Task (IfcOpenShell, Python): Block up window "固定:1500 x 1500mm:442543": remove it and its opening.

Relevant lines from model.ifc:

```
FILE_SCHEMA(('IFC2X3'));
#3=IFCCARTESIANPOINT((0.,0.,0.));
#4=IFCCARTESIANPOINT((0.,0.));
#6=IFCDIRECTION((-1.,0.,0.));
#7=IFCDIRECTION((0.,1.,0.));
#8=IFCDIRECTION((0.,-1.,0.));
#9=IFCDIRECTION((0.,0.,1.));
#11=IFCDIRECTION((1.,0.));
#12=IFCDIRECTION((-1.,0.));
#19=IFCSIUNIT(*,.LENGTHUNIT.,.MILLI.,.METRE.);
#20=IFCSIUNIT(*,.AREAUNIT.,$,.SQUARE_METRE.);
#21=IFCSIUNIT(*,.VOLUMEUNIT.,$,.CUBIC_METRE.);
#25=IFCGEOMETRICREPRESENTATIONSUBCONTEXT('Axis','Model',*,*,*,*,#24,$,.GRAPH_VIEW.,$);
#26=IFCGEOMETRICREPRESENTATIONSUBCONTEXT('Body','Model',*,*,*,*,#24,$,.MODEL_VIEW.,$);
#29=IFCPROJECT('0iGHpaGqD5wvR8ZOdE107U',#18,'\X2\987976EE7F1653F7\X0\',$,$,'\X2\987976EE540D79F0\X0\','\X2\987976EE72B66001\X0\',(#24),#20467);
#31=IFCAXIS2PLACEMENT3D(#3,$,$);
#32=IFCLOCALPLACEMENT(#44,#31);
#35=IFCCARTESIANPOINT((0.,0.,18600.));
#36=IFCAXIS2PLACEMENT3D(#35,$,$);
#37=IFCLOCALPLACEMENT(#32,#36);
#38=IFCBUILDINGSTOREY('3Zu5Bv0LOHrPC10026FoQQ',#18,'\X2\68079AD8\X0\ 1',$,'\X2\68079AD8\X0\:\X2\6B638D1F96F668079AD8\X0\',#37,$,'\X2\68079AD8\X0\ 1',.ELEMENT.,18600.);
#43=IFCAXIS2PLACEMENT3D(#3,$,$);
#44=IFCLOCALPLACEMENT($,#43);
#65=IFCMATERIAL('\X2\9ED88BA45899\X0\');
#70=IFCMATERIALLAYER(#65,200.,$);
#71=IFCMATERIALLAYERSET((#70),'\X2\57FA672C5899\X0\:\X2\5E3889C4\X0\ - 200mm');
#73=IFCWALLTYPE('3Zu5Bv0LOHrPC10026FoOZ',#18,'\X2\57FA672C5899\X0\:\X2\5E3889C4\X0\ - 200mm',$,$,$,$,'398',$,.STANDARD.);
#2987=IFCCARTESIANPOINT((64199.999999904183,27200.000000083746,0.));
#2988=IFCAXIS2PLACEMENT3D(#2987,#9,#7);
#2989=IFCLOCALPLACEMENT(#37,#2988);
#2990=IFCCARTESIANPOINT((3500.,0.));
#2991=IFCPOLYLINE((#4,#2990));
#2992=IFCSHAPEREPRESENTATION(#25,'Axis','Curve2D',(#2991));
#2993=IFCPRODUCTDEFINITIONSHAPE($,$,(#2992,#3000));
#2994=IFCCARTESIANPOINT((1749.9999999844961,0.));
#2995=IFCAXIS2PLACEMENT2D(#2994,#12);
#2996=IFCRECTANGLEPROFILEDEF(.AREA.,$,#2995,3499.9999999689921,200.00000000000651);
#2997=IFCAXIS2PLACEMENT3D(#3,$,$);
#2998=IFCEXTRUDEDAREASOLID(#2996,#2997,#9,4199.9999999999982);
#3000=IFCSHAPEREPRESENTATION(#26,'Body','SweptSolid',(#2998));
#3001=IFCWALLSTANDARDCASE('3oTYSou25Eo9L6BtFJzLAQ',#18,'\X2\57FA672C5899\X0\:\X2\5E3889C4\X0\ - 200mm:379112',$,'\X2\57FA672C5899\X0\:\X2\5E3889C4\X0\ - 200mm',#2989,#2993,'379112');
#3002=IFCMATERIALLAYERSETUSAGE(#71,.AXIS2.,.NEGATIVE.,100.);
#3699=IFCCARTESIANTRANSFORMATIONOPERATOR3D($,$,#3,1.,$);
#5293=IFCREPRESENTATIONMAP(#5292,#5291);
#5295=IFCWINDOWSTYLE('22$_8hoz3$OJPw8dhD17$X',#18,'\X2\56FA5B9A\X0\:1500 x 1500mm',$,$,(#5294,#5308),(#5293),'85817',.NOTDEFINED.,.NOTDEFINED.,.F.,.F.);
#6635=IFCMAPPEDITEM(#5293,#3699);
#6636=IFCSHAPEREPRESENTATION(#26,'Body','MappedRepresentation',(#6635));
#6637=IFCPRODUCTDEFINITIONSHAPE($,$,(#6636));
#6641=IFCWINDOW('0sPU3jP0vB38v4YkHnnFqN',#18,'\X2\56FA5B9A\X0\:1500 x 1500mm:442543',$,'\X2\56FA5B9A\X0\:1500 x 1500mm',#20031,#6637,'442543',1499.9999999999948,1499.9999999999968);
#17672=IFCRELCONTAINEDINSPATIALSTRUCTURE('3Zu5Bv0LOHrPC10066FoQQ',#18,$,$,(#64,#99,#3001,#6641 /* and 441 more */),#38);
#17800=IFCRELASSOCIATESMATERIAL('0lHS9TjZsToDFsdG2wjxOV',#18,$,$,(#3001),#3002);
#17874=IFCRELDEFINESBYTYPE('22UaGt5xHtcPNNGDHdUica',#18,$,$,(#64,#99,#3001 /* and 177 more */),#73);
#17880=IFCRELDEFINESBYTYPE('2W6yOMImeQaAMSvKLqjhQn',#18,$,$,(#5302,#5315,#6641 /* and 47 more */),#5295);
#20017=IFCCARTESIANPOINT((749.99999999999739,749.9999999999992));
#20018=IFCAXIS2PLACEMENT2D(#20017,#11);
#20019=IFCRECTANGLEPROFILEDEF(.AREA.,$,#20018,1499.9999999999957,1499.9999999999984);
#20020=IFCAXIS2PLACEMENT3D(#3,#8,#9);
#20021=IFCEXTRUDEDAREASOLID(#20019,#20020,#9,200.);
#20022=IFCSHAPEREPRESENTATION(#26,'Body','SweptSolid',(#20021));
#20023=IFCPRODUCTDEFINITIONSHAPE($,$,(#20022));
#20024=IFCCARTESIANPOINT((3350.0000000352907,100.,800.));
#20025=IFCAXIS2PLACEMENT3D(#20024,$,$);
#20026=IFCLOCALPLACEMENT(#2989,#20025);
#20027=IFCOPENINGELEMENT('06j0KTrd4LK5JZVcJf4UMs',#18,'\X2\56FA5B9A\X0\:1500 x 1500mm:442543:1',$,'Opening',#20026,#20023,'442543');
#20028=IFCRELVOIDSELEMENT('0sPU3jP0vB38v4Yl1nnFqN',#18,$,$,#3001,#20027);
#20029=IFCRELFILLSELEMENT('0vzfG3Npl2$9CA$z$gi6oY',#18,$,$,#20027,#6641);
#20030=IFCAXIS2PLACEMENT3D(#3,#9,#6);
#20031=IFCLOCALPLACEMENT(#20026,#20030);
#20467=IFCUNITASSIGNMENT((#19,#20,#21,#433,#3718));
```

```python
import ifcopenshell
import ifcopenshell.api.feature
import ifcopenshell.api.root
import ifcopenshell.geom
import ifcopenshell.util.shape

model = ifcopenshell.open("model.ifc")
settings = ifcopenshell.geom.settings()


def volume(element):
    """Net volume in cubic metres, openings subtracted."""
    shape = ifcopenshell.geom.create_shape(settings, element)
    return ifcopenshell.util.shape.get_volume(shape.geometry)


window = model.by_guid("0sPU3jP0vB38v4YkHnnFqN")
opening = window.FillsVoids[0].RelatingOpeningElement
wall = opening.VoidsElements[0].RelatingBuildingElement
before = volume(wall)

ifcopenshell.api.root.remove_product(model, product=window)
ifcopenshell.api.feature.remove_feature(model, feature=opening)

after = volume(wall)

print(f"wall volume {before:.3f} -> {after:.3f} m3")

model.write("model-out.ifc")
```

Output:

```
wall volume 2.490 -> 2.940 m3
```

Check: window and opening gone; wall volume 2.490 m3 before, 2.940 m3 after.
